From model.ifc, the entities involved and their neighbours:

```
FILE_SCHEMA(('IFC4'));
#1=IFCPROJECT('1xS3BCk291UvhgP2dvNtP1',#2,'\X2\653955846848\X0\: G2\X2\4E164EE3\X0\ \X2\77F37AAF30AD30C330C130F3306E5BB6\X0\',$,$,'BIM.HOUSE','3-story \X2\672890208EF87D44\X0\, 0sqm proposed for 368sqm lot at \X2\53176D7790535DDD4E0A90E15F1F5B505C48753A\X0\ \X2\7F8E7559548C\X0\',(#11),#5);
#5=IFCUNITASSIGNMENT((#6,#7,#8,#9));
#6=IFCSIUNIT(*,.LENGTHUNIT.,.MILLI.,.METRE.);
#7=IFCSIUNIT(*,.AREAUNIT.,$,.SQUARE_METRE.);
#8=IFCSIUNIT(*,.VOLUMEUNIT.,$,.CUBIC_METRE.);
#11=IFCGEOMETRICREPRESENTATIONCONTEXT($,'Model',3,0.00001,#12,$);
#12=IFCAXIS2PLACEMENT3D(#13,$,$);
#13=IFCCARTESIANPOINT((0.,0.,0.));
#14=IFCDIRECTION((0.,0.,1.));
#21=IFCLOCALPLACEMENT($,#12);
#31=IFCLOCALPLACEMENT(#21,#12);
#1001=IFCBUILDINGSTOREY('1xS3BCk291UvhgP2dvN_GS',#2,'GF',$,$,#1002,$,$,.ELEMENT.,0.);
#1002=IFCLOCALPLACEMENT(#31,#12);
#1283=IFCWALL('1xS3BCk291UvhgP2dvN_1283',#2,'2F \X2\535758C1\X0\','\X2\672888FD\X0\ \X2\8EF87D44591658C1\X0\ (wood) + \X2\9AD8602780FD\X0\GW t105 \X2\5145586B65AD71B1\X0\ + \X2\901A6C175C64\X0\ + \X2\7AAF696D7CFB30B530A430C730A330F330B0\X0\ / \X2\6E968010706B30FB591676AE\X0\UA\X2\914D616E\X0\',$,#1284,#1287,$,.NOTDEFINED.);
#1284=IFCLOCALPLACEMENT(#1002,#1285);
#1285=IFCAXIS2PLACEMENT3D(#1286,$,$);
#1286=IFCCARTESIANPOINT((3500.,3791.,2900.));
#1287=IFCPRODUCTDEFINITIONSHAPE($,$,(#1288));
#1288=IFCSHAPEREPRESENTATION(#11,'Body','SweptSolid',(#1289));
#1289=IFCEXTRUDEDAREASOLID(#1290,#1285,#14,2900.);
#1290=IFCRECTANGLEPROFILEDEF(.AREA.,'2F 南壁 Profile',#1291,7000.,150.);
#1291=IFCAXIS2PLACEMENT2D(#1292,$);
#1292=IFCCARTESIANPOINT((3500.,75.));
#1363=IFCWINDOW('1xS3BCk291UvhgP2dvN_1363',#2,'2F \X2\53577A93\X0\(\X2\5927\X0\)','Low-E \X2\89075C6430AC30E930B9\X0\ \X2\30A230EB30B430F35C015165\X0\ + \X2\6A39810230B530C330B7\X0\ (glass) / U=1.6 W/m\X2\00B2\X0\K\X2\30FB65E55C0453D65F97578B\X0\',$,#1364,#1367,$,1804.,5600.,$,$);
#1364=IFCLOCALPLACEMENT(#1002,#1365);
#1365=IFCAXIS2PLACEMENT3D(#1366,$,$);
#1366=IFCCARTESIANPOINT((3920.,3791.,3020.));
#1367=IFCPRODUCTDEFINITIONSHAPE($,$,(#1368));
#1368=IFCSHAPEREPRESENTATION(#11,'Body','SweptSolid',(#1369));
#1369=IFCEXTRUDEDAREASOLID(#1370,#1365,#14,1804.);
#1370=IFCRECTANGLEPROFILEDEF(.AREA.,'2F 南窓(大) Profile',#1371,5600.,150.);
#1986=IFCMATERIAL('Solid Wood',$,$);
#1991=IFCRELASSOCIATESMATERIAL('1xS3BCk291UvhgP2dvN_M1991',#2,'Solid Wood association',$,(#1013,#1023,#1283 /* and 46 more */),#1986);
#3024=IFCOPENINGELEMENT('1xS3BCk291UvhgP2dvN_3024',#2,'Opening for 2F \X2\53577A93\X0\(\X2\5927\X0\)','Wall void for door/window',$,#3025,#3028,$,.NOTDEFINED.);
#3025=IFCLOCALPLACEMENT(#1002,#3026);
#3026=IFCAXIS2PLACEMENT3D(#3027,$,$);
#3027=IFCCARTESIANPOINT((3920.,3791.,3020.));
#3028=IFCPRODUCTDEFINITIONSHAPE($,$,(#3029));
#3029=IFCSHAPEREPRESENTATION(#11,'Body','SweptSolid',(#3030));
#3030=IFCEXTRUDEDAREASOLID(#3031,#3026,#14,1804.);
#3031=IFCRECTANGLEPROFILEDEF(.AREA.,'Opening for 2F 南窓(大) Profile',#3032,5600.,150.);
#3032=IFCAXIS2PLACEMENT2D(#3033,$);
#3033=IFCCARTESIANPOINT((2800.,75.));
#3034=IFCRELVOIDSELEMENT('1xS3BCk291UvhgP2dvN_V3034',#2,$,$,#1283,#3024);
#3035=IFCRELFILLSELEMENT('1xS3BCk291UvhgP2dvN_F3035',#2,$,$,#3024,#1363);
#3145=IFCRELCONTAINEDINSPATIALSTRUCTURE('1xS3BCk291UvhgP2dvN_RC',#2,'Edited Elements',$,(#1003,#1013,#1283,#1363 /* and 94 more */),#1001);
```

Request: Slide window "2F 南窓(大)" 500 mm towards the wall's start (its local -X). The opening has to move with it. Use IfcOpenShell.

```python
import ifcopenshell
import ifcopenshell.api.geometry
import ifcopenshell.util.placement
import ifcopenshell.util.unit

model = ifcopenshell.open("model.ifc")
unit_scale = ifcopenshell.util.unit.calculate_unit_scale(model)

window = model.by_id(1363)
opening = window.FillsVoids[0].RelatingOpeningElement
wall = opening.VoidsElements[0].RelatingBuildingElement

wall_matrix = ifcopenshell.util.placement.get_local_placement(wall.ObjectPlacement)
shift = wall_matrix[:3, 0] * -0.5 / unit_scale
before = ifcopenshell.util.placement.get_local_placement(window.ObjectPlacement)[:3, 3].copy()

# The window is not placed relative to its opening, so move both.
for product in (opening, window):
    matrix = ifcopenshell.util.placement.get_local_placement(product.ObjectPlacement)
    matrix[:3, 3] += shift
    ifcopenshell.api.geometry.edit_object_placement(model, product=product, matrix=matrix, is_si=False)

after = ifcopenshell.util.placement.get_local_placement(window.ObjectPlacement)[:3, 3]
print("window moved by", (after - before).round(3) + 0.0)

model.write("model-out.ifc")
```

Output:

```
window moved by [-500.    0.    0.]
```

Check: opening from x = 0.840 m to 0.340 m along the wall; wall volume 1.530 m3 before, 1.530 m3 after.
